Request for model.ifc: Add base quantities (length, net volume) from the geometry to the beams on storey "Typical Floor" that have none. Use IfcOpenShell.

First a look at what the model holds.

```python
import ifcopenshell
import ifcopenshell.util.element
import ifcopenshell.util.unit

model = ifcopenshell.open("model.ifc")
print(model.schema)
for unit_type in ("LENGTHUNIT", "AREAUNIT", "VOLUMEUNIT"):
    print(unit_type, ifcopenshell.util.unit.calculate_unit_scale(model, unit_type))
storey = next(s for s in model.by_type("IfcBuildingStorey") if s.Name == "Typical Floor")
beams = [e for e in ifcopenshell.util.element.get_decomposition(storey) if e.is_a("IfcBeam")]
for e in sorted(beams, key=lambda e: e.id()):
    print(e.id(), e.is_a(), e.Name, list(ifcopenshell.util.element.get_psets(e, qtos_only=True)), sep=" | ")
```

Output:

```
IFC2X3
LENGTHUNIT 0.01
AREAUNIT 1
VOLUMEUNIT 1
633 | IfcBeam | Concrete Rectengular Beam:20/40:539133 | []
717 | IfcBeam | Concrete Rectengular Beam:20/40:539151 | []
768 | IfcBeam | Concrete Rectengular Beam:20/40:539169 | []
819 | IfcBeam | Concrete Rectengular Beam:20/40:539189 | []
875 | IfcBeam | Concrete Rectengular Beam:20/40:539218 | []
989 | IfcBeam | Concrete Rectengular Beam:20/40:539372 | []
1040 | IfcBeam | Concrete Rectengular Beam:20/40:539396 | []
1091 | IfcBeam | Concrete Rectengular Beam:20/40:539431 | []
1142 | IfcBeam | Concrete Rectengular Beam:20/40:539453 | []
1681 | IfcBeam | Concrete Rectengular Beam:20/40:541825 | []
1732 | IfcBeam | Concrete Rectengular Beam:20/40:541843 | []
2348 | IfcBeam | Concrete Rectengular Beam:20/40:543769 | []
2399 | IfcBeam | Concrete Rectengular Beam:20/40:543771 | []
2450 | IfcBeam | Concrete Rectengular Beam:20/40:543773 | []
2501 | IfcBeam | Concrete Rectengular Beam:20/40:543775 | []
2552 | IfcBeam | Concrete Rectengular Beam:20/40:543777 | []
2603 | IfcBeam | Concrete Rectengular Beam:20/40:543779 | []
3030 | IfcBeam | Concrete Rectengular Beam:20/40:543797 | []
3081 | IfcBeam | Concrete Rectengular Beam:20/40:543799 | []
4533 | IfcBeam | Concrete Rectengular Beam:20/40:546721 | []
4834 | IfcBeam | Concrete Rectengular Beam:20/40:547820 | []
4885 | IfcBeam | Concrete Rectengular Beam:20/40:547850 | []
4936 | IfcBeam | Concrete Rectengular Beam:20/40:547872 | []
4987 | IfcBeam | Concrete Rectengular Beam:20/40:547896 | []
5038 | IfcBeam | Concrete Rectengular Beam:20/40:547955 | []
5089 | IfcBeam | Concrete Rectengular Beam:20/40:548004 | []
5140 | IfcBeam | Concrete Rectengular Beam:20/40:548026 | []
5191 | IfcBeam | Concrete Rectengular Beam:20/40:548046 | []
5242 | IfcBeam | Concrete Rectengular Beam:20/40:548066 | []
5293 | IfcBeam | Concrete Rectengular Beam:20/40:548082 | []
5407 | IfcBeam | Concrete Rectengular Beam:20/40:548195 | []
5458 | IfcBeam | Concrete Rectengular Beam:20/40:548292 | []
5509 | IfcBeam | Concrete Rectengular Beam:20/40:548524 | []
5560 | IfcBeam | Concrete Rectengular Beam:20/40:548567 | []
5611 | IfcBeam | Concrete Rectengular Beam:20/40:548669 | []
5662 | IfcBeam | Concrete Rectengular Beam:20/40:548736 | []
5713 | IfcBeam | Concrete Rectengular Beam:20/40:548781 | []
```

```python
import ifcopenshell
import ifcopenshell.api.pset
import ifcopenshell.geom
import ifcopenshell.util.element
import ifcopenshell.util.shape
import ifcopenshell.util.unit

model = ifcopenshell.open("model.ifc")
unit_scale = ifcopenshell.util.unit.calculate_unit_scale(model)
volume_scale = ifcopenshell.util.unit.calculate_unit_scale(model, "VOLUMEUNIT")
settings = ifcopenshell.geom.settings()

storey = next(s for s in model.by_type("IfcBuildingStorey") if s.Name == "Typical Floor")
beams = [e for e in ifcopenshell.util.element.get_decomposition(storey) if e.is_a("IfcBeam")]

for e in sorted(beams, key=lambda e: e.id()):
    if ifcopenshell.util.element.get_psets(e, qtos_only=True, should_inherit=False):
        continue
    # Geometry comes back in metres, in the element's own axes.
    shape = ifcopenshell.geom.create_shape(settings, e)
    values = {
        "Length": ifcopenshell.util.shape.get_max_xyz(shape.geometry) / unit_scale,
        "NetVolume": ifcopenshell.util.shape.get_volume(shape.geometry) / volume_scale,
    }
    qto = ifcopenshell.api.pset.add_qto(model, product=e, name="BaseQuantities")
    ifcopenshell.api.pset.edit_qto(model, qto=qto, properties=values)
    print(e.id(), {k: round(v, 3) for k, v in values.items()})

model.write("model_edited.ifc")
```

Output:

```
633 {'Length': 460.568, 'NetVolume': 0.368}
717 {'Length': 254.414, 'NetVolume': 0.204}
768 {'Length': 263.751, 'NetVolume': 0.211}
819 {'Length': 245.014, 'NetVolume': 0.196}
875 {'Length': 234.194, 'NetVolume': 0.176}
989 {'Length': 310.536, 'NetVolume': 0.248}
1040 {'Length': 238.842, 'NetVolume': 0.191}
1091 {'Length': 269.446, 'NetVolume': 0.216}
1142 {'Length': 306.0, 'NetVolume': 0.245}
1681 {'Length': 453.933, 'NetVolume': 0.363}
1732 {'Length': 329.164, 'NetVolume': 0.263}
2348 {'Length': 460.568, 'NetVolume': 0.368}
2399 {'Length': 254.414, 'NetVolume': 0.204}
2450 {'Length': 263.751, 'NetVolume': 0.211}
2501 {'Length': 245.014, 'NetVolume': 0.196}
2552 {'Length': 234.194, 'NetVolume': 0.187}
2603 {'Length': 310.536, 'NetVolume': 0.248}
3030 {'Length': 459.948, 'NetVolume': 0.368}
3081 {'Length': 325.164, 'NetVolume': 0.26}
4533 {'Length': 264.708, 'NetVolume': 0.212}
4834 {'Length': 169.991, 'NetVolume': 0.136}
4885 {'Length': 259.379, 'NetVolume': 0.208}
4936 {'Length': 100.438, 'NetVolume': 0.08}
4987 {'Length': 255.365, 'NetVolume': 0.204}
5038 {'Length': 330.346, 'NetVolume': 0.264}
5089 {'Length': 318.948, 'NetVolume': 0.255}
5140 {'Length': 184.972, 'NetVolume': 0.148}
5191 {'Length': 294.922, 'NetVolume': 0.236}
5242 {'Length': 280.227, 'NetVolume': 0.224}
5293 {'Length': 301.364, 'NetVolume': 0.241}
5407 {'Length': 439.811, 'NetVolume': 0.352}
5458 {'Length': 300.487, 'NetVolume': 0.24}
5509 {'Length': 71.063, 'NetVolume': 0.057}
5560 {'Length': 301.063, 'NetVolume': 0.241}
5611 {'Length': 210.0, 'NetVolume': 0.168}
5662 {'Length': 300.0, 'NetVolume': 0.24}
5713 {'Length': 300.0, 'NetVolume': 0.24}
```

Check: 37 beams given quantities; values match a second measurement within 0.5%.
